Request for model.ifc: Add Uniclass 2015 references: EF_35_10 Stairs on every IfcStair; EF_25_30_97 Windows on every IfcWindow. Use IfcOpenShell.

First a look at what the model holds.

```python
import ifcopenshell

model = ifcopenshell.open("model.ifc")
print(model.schema)
print("classifications:", [c.Name for c in model.by_type("IfcClassification")])
for ifc_class in ("IfcDoor", "IfcRoof", "IfcStair", "IfcWall", "IfcWindow"):
    print(ifc_class, len(model.by_type(ifc_class)))
```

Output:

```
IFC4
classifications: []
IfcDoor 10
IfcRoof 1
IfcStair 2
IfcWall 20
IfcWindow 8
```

```python
import ifcopenshell
import ifcopenshell.api.classification

model = ifcopenshell.open("model.ifc")

system = ifcopenshell.api.classification.add_classification(model, classification="Uniclass 2015")

codes = {
    "IfcStair": ("EF_35_10", "Stairs"),
    "IfcWindow": ("EF_25_30_97", "Windows"),
}
for ifc_class, (code, name) in codes.items():
    products = model.by_type(ifc_class)
    ifcopenshell.api.classification.add_reference(
        model, products=products, classification=system, identification=code, name=name
    )
    print(code, len(products))

model.write("model_rev.ifc")
```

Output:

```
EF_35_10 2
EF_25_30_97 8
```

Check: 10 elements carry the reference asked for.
